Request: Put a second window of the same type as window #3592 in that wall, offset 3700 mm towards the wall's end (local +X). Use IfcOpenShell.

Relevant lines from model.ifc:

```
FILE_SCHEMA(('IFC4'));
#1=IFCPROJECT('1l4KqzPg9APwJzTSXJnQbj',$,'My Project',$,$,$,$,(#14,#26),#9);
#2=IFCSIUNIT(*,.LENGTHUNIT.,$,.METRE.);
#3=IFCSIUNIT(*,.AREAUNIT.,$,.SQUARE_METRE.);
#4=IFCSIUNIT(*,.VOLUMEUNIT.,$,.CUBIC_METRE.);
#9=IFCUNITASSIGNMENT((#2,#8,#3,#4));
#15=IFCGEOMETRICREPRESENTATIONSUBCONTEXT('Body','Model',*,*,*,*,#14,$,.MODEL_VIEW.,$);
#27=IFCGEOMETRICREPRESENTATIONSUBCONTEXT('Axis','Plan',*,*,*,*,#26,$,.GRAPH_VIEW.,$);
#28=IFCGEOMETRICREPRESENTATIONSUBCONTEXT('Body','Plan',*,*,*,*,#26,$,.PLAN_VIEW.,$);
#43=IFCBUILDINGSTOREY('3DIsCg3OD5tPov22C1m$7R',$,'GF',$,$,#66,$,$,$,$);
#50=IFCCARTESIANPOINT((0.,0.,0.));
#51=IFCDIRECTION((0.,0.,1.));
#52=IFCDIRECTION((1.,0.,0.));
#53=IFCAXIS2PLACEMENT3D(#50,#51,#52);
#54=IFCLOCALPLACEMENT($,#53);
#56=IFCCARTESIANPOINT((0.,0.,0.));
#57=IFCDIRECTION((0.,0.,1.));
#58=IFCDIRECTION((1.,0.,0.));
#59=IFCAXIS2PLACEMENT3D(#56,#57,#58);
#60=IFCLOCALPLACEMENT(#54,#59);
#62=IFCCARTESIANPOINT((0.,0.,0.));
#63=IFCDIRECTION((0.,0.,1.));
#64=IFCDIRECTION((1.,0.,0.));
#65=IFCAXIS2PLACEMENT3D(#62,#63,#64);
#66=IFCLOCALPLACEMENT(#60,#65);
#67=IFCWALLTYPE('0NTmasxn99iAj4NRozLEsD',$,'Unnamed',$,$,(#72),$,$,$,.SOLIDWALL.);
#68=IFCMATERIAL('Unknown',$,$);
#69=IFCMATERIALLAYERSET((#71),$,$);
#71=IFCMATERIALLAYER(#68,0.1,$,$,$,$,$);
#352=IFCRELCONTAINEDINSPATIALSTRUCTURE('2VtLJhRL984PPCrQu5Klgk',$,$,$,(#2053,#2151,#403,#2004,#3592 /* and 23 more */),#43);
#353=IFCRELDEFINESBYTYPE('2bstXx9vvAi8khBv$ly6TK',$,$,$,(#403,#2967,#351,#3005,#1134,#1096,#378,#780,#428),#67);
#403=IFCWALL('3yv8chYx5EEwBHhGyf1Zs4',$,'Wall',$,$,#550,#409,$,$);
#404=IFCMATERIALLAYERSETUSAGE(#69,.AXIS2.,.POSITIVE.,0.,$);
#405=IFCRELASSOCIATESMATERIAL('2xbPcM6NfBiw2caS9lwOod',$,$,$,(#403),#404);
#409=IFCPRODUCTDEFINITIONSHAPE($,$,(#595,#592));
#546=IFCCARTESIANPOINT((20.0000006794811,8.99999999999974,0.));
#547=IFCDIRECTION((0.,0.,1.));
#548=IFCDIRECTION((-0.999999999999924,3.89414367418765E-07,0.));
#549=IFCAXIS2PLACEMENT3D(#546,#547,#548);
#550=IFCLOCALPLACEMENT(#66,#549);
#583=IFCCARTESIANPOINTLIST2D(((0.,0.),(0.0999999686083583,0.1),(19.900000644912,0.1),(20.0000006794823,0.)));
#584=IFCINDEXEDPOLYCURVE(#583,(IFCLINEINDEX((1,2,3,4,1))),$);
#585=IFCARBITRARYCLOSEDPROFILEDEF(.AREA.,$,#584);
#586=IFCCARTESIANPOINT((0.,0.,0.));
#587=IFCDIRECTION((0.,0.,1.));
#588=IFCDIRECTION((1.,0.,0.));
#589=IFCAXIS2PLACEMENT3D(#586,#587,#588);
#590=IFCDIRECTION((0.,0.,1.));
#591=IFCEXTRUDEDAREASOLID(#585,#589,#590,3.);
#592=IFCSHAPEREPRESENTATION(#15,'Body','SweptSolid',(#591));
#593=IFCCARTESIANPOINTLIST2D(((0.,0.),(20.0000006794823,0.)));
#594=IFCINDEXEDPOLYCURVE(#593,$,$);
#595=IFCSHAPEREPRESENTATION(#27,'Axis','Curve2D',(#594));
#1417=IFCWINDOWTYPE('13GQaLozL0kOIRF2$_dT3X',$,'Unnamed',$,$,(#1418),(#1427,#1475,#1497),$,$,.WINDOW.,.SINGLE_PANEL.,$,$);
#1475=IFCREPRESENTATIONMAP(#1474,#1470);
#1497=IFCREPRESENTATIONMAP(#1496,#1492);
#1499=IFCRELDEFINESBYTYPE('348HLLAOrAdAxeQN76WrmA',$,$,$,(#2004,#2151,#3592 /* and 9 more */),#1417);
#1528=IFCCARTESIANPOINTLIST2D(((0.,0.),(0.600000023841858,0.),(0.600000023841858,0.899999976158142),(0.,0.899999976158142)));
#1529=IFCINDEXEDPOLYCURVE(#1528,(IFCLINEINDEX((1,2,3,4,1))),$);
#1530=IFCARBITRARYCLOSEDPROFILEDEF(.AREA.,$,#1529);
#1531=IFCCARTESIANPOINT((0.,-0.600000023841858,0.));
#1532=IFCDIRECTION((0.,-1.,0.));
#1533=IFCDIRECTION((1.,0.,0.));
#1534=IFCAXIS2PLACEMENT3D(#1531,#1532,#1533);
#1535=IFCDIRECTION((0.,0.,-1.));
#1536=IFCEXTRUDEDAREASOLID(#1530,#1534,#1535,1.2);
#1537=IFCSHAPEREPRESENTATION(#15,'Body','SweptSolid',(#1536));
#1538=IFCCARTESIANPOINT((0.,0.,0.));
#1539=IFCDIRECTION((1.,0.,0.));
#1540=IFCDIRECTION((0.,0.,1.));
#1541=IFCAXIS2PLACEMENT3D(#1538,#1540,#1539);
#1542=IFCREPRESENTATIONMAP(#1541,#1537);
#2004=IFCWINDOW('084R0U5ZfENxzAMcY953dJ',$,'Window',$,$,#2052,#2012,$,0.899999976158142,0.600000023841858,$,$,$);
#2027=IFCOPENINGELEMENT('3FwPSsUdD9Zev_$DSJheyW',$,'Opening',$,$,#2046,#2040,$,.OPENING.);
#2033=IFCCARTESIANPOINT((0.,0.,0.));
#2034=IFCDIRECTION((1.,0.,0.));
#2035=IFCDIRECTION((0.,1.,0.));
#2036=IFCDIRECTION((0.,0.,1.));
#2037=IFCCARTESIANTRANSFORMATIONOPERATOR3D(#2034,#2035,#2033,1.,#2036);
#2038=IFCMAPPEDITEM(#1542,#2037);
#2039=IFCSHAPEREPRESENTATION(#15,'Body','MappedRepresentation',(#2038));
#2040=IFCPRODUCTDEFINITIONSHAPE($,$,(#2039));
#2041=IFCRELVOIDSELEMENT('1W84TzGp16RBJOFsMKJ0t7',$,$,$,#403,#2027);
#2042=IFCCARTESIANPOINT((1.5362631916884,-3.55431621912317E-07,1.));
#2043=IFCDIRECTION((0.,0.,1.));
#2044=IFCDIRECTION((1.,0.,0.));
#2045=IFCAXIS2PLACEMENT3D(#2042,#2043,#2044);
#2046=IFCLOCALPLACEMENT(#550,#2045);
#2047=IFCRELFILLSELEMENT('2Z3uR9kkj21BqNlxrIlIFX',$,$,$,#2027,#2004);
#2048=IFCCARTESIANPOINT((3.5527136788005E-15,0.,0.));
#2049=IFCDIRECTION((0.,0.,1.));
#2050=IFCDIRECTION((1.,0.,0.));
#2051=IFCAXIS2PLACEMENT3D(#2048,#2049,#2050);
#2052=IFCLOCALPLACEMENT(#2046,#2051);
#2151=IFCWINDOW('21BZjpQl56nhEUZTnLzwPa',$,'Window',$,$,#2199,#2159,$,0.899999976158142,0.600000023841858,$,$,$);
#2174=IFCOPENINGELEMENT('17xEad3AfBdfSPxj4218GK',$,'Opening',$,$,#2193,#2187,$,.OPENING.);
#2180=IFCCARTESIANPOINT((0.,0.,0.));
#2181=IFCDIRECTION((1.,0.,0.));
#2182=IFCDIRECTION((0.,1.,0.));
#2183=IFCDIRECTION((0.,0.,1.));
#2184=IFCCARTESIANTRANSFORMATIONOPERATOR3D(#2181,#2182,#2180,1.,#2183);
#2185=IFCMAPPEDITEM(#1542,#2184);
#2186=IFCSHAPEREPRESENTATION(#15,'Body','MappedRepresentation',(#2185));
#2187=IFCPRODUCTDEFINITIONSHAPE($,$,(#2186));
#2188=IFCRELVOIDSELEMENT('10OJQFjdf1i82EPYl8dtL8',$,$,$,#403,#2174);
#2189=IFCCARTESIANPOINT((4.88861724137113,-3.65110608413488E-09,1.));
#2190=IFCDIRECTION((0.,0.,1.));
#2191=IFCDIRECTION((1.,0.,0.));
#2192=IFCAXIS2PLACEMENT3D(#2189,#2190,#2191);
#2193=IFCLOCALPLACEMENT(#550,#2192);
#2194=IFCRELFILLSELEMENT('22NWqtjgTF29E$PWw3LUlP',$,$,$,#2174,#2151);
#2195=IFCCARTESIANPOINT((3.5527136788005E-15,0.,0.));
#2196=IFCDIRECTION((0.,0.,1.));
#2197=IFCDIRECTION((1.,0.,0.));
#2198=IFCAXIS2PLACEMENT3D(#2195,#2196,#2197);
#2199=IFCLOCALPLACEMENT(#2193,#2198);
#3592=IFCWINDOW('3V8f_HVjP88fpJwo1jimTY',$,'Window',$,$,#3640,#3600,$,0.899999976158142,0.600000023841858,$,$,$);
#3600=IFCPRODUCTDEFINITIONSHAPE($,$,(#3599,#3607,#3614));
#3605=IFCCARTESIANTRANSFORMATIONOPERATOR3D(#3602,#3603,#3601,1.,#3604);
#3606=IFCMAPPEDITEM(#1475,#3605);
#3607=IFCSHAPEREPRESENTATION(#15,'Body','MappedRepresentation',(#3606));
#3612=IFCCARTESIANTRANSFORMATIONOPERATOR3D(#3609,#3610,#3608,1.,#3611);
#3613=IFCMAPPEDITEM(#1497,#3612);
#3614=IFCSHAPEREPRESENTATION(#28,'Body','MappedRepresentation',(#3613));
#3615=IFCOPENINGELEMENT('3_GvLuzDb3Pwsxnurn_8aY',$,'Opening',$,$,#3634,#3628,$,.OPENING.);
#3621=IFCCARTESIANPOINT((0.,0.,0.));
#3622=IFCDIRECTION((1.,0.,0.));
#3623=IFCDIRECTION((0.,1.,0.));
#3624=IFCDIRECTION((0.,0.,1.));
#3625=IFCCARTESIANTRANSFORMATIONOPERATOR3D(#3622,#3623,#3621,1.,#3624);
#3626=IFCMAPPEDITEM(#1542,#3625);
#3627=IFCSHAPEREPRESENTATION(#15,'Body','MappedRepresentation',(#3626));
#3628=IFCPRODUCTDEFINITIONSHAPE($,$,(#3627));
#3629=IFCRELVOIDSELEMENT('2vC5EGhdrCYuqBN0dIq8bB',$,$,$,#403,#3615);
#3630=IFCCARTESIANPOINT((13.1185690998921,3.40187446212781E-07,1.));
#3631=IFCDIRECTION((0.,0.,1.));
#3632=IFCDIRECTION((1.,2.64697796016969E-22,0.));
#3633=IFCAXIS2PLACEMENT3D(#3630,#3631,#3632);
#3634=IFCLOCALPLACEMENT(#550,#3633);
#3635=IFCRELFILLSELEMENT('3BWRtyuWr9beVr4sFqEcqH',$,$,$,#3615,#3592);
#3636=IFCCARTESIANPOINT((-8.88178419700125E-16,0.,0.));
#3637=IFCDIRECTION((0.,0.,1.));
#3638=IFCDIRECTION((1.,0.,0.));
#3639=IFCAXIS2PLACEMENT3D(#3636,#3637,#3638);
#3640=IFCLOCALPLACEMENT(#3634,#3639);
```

```python
import ifcopenshell
import ifcopenshell.api.feature
import ifcopenshell.api.geometry
import ifcopenshell.api.root
import ifcopenshell.geom
import ifcopenshell.util.element
import ifcopenshell.util.placement
import ifcopenshell.util.shape
import ifcopenshell.util.unit

model = ifcopenshell.open("model.ifc")
unit_scale = ifcopenshell.util.unit.calculate_unit_scale(model)
settings = ifcopenshell.geom.settings()


def volume(element):
    """Net volume in cubic metres, openings subtracted."""
    shape = ifcopenshell.geom.create_shape(settings, element)
    return ifcopenshell.util.shape.get_volume(shape.geometry)


window = model.by_guid("3V8f_HVjP88fpJwo1jimTY")
opening = window.FillsVoids[0].RelatingOpeningElement
wall = opening.VoidsElements[0].RelatingBuildingElement
before = volume(wall)
shift = ifcopenshell.util.placement.get_local_placement(wall.ObjectPlacement)[:3, 0] * 3.7 / unit_scale

# copy_class copies the void relationship, type, container and properties, but no geometry.
new_opening = ifcopenshell.api.root.copy_class(model, product=opening)
new_opening.Representation = ifcopenshell.util.element.copy_deep(
    model, opening.Representation, exclude=["IfcGeometricRepresentationContext", "IfcRepresentationMap"]
)
new_window = ifcopenshell.api.root.copy_class(model, product=window)
new_window.Representation = ifcopenshell.util.element.copy_deep(
    model, window.Representation, exclude=["IfcGeometricRepresentationContext", "IfcRepresentationMap"]
)
ifcopenshell.api.feature.add_filling(model, opening=new_opening, element=new_window)

for old, new in ((opening, new_opening), (window, new_window)):
    matrix = ifcopenshell.util.placement.get_local_placement(old.ObjectPlacement)
    matrix[:3, 3] += shift
    ifcopenshell.api.geometry.edit_object_placement(model, product=new, matrix=matrix, is_si=False)

after = volume(wall)

print(f"wall volume {before:.3f} -> {after:.3f} m3")

model.write("model_rev.ifc")
```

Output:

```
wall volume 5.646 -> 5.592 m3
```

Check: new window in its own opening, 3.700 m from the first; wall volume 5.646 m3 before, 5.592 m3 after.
